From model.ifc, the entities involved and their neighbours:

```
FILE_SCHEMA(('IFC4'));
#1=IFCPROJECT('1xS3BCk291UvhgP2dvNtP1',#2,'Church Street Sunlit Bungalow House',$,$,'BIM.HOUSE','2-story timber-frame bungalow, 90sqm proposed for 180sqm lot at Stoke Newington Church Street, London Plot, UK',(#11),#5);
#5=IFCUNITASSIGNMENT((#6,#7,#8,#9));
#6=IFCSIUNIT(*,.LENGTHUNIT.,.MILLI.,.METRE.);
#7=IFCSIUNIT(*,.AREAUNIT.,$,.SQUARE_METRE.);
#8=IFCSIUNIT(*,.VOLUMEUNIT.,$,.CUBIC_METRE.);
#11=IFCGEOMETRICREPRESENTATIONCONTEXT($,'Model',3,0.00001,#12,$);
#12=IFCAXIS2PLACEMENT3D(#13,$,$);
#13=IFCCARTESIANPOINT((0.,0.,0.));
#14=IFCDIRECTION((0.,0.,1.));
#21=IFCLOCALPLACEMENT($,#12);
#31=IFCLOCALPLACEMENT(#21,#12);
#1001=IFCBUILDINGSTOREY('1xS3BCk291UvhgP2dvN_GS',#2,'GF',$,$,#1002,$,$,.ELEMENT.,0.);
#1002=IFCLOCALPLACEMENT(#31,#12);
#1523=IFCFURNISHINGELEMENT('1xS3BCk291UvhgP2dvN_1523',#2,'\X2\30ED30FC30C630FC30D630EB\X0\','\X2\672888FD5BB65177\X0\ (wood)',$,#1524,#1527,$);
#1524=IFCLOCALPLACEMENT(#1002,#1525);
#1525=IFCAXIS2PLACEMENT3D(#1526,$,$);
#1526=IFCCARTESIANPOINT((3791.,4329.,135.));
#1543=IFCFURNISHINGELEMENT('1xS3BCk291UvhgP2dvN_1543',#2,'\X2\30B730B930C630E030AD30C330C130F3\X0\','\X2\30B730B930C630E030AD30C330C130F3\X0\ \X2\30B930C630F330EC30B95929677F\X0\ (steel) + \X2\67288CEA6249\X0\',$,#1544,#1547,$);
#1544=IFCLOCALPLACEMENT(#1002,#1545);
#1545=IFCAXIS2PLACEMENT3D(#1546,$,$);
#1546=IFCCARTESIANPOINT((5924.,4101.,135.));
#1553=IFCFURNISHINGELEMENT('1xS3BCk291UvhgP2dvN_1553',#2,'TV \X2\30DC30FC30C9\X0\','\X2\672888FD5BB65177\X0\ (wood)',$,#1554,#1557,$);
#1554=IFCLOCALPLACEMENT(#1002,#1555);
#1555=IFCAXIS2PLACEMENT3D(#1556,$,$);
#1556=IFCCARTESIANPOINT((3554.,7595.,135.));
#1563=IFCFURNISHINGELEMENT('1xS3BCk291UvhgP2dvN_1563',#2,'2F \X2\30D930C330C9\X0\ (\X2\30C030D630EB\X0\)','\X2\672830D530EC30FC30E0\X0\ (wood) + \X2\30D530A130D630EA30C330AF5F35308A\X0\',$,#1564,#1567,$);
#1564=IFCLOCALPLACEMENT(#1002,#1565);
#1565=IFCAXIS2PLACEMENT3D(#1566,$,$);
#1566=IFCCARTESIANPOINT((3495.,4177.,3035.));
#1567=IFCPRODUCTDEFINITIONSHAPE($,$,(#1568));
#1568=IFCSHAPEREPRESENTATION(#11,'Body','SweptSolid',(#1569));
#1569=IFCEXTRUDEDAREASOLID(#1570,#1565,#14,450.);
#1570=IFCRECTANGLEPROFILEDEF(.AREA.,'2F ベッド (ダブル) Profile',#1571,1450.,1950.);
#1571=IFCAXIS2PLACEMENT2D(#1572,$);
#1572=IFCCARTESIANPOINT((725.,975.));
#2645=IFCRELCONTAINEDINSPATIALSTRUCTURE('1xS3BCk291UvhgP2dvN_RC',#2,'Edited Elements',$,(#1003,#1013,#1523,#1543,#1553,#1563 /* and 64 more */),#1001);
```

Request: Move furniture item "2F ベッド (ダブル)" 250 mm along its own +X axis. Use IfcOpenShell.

```python
import ifcopenshell
import ifcopenshell.api.geometry
import ifcopenshell.util.placement
import ifcopenshell.util.unit

model = ifcopenshell.open("model.ifc")
unit_scale = ifcopenshell.util.unit.calculate_unit_scale(model)

item = model.by_guid("1xS3BCk291UvhgP2dvN_1563")
matrix = ifcopenshell.util.placement.get_local_placement(item.ObjectPlacement)
matrix[:3, 3] += matrix[:3, 0] * 0.25 / unit_scale
ifcopenshell.api.geometry.edit_object_placement(model, product=item, matrix=matrix, is_si=False)

print(ifcopenshell.util.placement.get_local_placement(item.ObjectPlacement).round(3) + 0.0)

model.write("model_rev.ifc")
```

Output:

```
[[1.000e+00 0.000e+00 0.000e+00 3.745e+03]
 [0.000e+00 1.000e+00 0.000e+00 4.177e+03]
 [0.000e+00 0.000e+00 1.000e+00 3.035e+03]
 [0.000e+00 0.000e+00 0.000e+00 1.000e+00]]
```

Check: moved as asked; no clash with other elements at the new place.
